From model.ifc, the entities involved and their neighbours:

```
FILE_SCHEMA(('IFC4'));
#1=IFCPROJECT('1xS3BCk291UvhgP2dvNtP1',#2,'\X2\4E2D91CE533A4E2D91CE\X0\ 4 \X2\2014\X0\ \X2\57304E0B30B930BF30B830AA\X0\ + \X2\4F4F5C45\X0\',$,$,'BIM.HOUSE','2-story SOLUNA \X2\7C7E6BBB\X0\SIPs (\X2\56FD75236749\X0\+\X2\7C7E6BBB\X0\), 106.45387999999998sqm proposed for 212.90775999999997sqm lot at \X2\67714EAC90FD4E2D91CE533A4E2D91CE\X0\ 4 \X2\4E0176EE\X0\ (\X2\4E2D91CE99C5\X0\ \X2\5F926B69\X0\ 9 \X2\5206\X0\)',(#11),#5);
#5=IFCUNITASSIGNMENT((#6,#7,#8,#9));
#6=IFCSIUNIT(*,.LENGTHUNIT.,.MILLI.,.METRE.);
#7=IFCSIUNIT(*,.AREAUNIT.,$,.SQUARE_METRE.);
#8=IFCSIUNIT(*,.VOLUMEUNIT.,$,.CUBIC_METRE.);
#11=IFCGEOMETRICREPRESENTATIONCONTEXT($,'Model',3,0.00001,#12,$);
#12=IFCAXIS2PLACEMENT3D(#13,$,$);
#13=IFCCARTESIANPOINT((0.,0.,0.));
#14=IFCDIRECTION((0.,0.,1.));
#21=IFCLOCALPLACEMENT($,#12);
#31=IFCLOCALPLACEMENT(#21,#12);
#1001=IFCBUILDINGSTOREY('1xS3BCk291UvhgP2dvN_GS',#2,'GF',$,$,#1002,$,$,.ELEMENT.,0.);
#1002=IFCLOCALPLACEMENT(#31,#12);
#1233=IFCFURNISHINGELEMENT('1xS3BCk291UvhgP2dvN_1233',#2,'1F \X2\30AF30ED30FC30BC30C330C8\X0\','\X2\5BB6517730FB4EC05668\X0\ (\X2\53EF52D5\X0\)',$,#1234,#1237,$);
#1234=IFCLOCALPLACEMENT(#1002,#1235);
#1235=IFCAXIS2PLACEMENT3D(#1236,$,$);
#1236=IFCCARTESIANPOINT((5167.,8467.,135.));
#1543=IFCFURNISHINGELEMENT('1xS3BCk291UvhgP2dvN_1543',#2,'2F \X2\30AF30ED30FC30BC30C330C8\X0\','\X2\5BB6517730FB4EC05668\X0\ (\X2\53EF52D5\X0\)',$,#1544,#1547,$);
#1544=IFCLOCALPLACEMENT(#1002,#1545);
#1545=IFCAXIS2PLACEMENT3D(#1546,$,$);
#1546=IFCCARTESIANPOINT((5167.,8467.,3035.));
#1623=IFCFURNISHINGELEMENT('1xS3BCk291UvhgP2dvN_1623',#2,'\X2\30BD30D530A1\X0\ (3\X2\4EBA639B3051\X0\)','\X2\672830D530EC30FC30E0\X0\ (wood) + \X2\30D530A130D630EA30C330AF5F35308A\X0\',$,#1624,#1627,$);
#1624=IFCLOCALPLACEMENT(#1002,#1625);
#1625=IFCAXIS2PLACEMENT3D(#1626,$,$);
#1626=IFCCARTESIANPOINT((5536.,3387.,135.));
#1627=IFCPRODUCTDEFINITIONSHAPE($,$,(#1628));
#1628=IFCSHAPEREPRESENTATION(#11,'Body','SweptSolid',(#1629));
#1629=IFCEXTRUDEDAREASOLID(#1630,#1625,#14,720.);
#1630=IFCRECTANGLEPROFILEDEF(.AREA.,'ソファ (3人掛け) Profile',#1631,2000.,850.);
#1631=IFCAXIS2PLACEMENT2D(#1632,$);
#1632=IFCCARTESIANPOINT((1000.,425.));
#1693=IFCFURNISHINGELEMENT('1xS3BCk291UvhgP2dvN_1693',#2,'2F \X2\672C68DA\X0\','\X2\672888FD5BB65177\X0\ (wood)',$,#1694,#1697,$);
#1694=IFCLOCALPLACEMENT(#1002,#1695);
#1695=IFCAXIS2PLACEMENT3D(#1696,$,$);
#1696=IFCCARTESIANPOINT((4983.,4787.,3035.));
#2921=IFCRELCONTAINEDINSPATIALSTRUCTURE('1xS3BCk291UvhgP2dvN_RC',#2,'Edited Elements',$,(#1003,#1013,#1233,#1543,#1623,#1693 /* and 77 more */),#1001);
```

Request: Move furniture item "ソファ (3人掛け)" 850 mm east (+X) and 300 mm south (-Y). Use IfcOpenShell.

```python
import ifcopenshell
import ifcopenshell.api.geometry
import ifcopenshell.util.placement
import ifcopenshell.util.unit

model = ifcopenshell.open("model.ifc")
unit_scale = ifcopenshell.util.unit.calculate_unit_scale(model)

item = model.by_guid("1xS3BCk291UvhgP2dvN_1623")
matrix = ifcopenshell.util.placement.get_local_placement(item.ObjectPlacement)
matrix[0, 3] += 0.85 / unit_scale
matrix[1, 3] -= 0.3 / unit_scale
ifcopenshell.api.geometry.edit_object_placement(model, product=item, matrix=matrix, is_si=False)

print(ifcopenshell.util.placement.get_local_placement(item.ObjectPlacement).round(3) + 0.0)

model.write("model_updated.ifc")
```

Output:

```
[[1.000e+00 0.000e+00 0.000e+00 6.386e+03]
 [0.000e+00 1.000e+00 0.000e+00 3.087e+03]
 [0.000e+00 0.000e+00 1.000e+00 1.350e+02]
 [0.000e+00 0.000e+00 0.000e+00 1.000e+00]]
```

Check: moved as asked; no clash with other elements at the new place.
